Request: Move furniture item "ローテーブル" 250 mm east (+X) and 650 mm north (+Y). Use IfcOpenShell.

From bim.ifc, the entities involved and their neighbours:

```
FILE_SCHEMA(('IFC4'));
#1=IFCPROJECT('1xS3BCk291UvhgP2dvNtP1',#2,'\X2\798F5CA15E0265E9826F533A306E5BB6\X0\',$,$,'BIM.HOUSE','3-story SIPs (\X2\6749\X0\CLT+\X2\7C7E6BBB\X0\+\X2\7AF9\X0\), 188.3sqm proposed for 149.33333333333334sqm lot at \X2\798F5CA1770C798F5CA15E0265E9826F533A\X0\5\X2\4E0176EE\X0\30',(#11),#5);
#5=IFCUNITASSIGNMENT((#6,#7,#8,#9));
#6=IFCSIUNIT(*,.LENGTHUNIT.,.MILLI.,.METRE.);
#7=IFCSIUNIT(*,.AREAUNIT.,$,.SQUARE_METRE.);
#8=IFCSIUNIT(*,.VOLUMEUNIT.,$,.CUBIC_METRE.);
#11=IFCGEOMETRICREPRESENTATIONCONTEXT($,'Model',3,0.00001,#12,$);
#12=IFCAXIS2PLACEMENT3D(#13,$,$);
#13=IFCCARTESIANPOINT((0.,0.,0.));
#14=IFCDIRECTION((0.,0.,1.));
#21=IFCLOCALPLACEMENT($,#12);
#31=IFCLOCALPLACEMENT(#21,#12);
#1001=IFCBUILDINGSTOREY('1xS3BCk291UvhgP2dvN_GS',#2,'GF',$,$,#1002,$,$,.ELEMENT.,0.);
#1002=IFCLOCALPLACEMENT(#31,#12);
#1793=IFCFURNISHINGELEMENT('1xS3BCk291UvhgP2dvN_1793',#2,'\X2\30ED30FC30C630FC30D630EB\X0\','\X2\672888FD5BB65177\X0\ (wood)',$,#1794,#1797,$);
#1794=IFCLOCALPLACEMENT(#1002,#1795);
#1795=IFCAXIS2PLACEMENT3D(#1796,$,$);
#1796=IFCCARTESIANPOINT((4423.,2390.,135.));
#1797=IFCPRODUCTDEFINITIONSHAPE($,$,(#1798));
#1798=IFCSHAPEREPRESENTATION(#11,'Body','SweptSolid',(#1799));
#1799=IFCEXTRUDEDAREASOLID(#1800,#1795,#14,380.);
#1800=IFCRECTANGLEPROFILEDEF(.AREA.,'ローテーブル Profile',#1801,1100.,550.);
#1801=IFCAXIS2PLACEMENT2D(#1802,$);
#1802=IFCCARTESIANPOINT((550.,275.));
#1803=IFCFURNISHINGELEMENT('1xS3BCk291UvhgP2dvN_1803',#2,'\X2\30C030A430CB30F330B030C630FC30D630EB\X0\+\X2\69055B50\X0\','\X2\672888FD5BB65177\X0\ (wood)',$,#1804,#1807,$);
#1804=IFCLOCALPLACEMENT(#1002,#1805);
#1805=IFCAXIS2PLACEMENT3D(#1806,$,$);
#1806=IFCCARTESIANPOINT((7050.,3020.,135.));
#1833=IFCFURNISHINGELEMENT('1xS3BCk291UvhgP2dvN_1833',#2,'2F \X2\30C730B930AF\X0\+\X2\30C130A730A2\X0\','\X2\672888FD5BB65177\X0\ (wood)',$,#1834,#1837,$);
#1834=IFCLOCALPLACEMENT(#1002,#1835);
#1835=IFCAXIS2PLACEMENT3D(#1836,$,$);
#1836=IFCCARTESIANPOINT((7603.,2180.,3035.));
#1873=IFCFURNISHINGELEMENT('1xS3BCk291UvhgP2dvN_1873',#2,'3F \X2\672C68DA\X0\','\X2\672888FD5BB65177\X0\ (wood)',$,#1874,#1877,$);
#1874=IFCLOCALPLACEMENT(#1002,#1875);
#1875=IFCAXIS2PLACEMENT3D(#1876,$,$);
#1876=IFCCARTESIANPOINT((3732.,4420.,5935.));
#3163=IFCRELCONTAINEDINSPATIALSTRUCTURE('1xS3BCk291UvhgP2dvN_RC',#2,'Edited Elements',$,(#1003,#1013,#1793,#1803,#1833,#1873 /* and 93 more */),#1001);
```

```python
import ifcopenshell
import ifcopenshell.api.geometry
import ifcopenshell.util.placement

model = ifcopenshell.open("bim.ifc")

item = model.by_id(1793)
matrix = ifcopenshell.util.placement.get_local_placement(item.ObjectPlacement)
matrix[0, 3] += 250.0
matrix[1, 3] += 650.0
ifcopenshell.api.geometry.edit_object_placement(model, product=item, matrix=matrix, is_si=False)

print(ifcopenshell.util.placement.get_local_placement(item.ObjectPlacement).round(3) + 0.0)

model.write("bim_v2.ifc")
```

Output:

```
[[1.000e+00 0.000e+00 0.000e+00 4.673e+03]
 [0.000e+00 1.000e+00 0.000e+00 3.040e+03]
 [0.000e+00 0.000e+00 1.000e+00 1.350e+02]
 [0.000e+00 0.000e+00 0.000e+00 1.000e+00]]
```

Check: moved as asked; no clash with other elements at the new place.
